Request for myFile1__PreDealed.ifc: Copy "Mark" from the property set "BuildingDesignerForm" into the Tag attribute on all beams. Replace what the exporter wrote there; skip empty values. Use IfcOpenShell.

First a look at what the model holds.

```python
import ifcopenshell
import ifcopenshell.util.element

model = ifcopenshell.open("myFile1__PreDealed.ifc")
print(model.schema)
beams = model.by_type("IfcBeam")
print(len(beams), "beams")
for e in beams[:8]:
    source = ifcopenshell.util.element.get_pset(e, "BuildingDesignerForm", "Mark")
    target = e.Tag
    print(e.id(), repr(source), repr(target), sep=" | ")
```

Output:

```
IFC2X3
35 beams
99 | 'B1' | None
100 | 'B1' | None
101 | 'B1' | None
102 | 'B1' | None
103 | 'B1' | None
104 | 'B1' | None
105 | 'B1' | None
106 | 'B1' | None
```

```python
import ifcopenshell
import ifcopenshell.util.element

model = ifcopenshell.open("myFile1__PreDealed.ifc")

count = 0
for e in model.by_type("IfcBeam"):
    value = ifcopenshell.util.element.get_pset(e, "BuildingDesignerForm", "Mark")
    current = e.Tag
    if not value or not value.strip() or current == value:
        continue
    e.Tag = value
    count += 1

print(count, "beams updated")

model.write("myFile1__PreDealed_rev.ifc")
```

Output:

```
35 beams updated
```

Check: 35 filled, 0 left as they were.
